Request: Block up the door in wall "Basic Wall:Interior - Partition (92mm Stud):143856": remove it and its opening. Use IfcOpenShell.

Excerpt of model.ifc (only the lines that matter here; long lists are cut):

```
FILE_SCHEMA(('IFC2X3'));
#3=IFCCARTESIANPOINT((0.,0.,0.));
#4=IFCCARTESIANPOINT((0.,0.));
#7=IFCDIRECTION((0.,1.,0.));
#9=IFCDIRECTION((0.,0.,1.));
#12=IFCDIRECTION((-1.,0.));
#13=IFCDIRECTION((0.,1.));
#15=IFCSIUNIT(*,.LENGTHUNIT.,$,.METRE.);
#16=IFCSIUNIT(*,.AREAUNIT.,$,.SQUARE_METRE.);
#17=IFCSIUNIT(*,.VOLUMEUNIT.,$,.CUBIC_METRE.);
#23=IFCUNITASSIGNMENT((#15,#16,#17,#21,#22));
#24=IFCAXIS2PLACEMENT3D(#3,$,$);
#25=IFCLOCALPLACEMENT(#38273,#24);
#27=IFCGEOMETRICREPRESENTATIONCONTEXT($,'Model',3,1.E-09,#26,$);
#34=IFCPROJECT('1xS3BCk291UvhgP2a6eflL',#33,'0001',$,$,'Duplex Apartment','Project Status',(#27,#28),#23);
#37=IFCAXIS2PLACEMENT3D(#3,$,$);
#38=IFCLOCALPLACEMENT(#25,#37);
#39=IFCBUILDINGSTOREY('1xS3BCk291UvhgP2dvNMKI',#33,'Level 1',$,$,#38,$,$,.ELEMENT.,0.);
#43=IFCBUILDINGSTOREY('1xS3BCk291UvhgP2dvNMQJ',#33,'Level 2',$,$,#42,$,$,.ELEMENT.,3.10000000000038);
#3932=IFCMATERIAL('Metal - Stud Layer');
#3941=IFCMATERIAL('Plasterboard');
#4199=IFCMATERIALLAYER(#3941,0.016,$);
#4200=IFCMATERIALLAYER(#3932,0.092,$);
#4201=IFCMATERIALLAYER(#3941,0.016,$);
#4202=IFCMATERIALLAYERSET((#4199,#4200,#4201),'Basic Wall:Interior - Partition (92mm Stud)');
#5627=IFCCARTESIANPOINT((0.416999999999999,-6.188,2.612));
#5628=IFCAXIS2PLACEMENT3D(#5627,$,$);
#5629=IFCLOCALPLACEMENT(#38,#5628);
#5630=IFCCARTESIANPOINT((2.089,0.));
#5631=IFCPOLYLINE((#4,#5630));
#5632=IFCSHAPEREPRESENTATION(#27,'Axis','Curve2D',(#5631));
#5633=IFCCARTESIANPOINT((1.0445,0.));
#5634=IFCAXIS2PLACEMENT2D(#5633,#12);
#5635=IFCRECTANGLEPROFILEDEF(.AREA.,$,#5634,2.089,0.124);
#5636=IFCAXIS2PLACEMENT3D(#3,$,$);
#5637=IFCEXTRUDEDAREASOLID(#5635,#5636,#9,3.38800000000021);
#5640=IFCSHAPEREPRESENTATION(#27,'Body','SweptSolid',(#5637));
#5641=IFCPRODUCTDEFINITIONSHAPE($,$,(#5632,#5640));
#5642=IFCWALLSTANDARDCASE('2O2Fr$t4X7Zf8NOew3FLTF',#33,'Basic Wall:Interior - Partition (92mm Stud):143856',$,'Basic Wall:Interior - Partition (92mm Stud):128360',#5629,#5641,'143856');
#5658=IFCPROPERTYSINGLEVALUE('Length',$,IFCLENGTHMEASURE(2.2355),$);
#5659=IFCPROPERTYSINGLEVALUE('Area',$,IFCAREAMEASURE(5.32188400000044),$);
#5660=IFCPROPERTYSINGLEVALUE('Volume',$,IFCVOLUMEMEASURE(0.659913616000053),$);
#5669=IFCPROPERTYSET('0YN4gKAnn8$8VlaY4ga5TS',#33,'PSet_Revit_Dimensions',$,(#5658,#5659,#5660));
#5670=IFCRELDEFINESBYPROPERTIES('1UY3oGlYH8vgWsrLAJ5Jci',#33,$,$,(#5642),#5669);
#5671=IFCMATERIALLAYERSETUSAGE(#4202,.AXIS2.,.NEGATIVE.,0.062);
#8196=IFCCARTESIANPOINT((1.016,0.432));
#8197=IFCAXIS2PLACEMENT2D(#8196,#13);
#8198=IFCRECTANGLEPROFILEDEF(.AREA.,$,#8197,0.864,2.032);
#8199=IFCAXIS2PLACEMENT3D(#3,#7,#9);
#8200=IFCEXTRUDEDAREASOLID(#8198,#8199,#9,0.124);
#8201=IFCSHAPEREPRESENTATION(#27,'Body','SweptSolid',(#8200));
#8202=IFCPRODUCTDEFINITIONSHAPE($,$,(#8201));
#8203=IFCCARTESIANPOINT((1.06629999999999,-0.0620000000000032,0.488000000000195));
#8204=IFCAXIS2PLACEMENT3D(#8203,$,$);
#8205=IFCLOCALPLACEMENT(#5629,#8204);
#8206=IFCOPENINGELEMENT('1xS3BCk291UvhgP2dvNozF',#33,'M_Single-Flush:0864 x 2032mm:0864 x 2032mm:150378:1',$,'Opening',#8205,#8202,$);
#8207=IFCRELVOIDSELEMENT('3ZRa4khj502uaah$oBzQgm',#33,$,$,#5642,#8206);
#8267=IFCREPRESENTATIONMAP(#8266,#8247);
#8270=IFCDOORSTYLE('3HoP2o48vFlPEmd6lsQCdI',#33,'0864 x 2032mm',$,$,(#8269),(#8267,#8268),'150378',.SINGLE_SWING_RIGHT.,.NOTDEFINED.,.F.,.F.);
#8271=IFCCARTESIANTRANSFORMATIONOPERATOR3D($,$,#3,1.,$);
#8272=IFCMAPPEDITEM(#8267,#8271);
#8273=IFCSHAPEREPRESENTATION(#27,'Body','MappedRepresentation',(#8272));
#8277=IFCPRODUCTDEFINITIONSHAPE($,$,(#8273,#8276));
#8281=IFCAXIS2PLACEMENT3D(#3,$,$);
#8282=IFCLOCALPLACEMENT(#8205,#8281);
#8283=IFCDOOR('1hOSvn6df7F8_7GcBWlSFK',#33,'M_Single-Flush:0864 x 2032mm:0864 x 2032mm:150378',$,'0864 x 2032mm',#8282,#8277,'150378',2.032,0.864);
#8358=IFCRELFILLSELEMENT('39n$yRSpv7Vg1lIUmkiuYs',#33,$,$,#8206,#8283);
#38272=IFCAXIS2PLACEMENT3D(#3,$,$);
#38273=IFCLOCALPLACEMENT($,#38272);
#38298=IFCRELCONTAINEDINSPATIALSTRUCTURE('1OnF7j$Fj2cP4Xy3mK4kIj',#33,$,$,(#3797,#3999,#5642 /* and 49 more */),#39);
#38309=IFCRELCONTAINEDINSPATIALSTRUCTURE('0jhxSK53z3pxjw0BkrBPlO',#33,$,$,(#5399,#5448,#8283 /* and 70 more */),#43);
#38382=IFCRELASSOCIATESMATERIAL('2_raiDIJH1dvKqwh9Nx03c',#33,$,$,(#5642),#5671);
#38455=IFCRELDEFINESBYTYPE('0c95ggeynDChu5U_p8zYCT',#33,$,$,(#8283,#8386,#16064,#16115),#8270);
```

```python
import ifcopenshell
import ifcopenshell.api.feature
import ifcopenshell.api.pset
import ifcopenshell.api.root
import ifcopenshell.geom
import ifcopenshell.util.element
import ifcopenshell.util.shape
import ifcopenshell.util.unit

model = ifcopenshell.open("model.ifc")
area_scale = ifcopenshell.util.unit.calculate_unit_scale(model, "AREAUNIT")
volume_scale = ifcopenshell.util.unit.calculate_unit_scale(model, "VOLUMEUNIT")
settings = ifcopenshell.geom.settings()


def volume(element):
    """Net volume in cubic metres, openings subtracted."""
    shape = ifcopenshell.geom.create_shape(settings, element)
    return ifcopenshell.util.shape.get_volume(shape.geometry)


door = model.by_guid("1hOSvn6df7F8_7GcBWlSFK")
opening = door.FillsVoids[0].RelatingOpeningElement
wall = opening.VoidsElements[0].RelatingBuildingElement
before = volume(wall)

ifcopenshell.api.root.remove_product(model, product=door)
ifcopenshell.api.feature.remove_feature(model, feature=opening)

after = volume(wall)
thickness = 0.124  # wall thickness in metres

# Update the wall's stored quantities.
pset = model.by_id(ifcopenshell.util.element.get_pset(wall, "PSet_Revit_Dimensions", should_inherit=False)["id"])
ifcopenshell.api.pset.edit_pset(model, pset=pset, properties={
    "Area": model.create_entity("IfcAreaMeasure", after / thickness / area_scale),
    "Volume": model.create_entity("IfcVolumeMeasure", after / volume_scale),
})

print(f"wall volume {before:.3f} -> {after:.3f} m3")

model.write("model-out.ifc")
```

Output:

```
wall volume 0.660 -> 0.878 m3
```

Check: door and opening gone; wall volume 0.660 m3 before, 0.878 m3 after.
